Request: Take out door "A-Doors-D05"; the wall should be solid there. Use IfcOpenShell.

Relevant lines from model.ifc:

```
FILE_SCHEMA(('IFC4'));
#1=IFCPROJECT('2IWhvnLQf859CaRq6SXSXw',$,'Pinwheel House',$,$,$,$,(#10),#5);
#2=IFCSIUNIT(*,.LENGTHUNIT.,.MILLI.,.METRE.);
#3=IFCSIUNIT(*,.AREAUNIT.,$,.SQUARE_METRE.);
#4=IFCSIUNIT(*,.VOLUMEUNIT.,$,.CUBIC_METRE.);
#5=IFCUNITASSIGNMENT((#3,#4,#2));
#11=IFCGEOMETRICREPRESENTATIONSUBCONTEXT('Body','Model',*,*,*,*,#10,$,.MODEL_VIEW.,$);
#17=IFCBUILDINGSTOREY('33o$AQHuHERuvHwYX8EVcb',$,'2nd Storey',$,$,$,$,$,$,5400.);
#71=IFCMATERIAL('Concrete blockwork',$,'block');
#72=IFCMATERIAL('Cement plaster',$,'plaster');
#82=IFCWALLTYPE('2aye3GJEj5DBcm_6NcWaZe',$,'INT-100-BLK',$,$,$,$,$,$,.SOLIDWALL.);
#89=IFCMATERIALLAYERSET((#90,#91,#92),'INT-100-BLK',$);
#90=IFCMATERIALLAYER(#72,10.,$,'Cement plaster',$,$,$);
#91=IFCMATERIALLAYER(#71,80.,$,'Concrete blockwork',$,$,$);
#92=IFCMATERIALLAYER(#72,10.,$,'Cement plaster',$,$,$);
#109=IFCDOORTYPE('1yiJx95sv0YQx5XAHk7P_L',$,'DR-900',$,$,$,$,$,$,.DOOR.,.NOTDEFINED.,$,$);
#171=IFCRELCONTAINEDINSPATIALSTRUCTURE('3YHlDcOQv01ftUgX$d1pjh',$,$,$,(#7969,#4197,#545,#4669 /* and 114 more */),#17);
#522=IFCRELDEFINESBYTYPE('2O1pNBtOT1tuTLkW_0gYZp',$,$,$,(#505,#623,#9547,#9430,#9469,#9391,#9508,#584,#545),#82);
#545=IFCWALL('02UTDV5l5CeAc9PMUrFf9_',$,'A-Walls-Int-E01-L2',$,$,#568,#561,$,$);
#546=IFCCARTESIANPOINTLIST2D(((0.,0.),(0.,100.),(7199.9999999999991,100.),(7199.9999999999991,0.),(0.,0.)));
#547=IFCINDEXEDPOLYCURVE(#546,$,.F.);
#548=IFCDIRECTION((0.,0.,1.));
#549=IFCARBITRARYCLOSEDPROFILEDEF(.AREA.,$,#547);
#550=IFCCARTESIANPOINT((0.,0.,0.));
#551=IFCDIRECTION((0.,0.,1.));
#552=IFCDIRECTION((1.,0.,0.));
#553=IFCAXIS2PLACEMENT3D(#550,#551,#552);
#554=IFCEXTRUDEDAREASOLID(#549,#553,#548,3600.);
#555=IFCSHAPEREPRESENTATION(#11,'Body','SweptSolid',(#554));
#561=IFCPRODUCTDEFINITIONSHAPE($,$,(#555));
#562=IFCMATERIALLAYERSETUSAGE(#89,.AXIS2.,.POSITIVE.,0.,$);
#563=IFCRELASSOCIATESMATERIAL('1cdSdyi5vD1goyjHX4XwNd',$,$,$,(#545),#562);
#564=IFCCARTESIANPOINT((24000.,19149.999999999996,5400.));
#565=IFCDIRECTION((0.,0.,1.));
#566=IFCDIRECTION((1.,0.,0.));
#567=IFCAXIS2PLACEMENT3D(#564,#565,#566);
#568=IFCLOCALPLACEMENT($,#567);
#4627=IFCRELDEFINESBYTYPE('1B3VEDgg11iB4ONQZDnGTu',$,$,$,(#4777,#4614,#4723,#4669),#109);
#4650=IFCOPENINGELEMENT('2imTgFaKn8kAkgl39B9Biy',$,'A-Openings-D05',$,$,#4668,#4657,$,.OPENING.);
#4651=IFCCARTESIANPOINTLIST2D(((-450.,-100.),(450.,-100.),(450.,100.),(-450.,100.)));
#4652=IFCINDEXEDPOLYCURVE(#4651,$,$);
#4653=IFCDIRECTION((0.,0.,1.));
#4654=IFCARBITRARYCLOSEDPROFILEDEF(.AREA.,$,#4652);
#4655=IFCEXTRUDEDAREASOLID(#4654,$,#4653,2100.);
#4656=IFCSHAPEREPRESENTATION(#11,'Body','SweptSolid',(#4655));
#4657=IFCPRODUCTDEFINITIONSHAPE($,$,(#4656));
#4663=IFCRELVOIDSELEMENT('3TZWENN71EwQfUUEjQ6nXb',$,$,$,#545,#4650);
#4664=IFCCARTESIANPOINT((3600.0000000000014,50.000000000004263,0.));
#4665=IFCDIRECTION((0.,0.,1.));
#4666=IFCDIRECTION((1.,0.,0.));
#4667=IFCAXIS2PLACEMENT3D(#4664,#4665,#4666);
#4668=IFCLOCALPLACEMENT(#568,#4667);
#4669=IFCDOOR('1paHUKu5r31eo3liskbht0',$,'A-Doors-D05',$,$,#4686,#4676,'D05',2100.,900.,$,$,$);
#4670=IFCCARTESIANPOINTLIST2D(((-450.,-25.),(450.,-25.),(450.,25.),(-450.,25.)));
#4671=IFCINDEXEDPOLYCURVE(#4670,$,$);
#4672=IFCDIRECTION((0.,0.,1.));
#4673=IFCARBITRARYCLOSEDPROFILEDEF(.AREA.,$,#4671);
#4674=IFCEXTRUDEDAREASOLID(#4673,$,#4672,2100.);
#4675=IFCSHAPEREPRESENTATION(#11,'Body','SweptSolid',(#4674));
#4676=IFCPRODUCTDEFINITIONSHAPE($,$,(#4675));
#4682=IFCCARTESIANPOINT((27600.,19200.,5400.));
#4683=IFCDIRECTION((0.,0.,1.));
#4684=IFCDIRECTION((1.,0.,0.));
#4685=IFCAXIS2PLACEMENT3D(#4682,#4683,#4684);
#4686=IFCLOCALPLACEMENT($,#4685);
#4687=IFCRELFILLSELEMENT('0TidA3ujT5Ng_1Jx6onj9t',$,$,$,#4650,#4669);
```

```python
import ifcopenshell
import ifcopenshell.api.feature
import ifcopenshell.api.root
import ifcopenshell.geom
import ifcopenshell.util.shape

model = ifcopenshell.open("model.ifc")
settings = ifcopenshell.geom.settings()


def volume(element):
    """Net volume in cubic metres, openings subtracted."""
    shape = ifcopenshell.geom.create_shape(settings, element)
    return ifcopenshell.util.shape.get_volume(shape.geometry)


door = model.by_guid("1paHUKu5r31eo3liskbht0")
opening = door.FillsVoids[0].RelatingOpeningElement
wall = opening.VoidsElements[0].RelatingBuildingElement
before = volume(wall)

ifcopenshell.api.root.remove_product(model, product=door)
ifcopenshell.api.feature.remove_feature(model, feature=opening)

after = volume(wall)

print(f"wall volume {before:.3f} -> {after:.3f} m3")

model.write("model_v2.ifc")
```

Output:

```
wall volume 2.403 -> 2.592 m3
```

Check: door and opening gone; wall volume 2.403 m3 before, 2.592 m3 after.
